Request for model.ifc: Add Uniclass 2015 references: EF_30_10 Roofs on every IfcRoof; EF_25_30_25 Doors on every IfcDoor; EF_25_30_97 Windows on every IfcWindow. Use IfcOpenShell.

First a look at what the model holds.

```python
import ifcopenshell

model = ifcopenshell.open("model.ifc")
print(model.schema)
print("classifications:", [c.Name for c in model.by_type("IfcClassification")])
for ifc_class in ("IfcDoor", "IfcRoof", "IfcStair", "IfcWall", "IfcWindow"):
    print(ifc_class, len(model.by_type(ifc_class)))
```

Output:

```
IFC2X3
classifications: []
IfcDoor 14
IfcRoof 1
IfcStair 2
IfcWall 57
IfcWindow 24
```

```python
import ifcopenshell
import ifcopenshell.api.classification

model = ifcopenshell.open("model.ifc")

# IFC2X3 requires Source and Edition and has no link from the project to the system.
system = model.create_entity("IfcClassification", Source="NBS", Edition="2015", Name="Uniclass 2015")

codes = {
    "IfcRoof": ("EF_30_10", "Roofs"),
    "IfcDoor": ("EF_25_30_25", "Doors"),
    "IfcWindow": ("EF_25_30_97", "Windows"),
}
for ifc_class, (code, name) in codes.items():
    products = model.by_type(ifc_class)
    ifcopenshell.api.classification.add_reference(
        model, products=products, classification=system, identification=code, name=name
    )
    print(code, len(products))

model.write("model-out.ifc")
```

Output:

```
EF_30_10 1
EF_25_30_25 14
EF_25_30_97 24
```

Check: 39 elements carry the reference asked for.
